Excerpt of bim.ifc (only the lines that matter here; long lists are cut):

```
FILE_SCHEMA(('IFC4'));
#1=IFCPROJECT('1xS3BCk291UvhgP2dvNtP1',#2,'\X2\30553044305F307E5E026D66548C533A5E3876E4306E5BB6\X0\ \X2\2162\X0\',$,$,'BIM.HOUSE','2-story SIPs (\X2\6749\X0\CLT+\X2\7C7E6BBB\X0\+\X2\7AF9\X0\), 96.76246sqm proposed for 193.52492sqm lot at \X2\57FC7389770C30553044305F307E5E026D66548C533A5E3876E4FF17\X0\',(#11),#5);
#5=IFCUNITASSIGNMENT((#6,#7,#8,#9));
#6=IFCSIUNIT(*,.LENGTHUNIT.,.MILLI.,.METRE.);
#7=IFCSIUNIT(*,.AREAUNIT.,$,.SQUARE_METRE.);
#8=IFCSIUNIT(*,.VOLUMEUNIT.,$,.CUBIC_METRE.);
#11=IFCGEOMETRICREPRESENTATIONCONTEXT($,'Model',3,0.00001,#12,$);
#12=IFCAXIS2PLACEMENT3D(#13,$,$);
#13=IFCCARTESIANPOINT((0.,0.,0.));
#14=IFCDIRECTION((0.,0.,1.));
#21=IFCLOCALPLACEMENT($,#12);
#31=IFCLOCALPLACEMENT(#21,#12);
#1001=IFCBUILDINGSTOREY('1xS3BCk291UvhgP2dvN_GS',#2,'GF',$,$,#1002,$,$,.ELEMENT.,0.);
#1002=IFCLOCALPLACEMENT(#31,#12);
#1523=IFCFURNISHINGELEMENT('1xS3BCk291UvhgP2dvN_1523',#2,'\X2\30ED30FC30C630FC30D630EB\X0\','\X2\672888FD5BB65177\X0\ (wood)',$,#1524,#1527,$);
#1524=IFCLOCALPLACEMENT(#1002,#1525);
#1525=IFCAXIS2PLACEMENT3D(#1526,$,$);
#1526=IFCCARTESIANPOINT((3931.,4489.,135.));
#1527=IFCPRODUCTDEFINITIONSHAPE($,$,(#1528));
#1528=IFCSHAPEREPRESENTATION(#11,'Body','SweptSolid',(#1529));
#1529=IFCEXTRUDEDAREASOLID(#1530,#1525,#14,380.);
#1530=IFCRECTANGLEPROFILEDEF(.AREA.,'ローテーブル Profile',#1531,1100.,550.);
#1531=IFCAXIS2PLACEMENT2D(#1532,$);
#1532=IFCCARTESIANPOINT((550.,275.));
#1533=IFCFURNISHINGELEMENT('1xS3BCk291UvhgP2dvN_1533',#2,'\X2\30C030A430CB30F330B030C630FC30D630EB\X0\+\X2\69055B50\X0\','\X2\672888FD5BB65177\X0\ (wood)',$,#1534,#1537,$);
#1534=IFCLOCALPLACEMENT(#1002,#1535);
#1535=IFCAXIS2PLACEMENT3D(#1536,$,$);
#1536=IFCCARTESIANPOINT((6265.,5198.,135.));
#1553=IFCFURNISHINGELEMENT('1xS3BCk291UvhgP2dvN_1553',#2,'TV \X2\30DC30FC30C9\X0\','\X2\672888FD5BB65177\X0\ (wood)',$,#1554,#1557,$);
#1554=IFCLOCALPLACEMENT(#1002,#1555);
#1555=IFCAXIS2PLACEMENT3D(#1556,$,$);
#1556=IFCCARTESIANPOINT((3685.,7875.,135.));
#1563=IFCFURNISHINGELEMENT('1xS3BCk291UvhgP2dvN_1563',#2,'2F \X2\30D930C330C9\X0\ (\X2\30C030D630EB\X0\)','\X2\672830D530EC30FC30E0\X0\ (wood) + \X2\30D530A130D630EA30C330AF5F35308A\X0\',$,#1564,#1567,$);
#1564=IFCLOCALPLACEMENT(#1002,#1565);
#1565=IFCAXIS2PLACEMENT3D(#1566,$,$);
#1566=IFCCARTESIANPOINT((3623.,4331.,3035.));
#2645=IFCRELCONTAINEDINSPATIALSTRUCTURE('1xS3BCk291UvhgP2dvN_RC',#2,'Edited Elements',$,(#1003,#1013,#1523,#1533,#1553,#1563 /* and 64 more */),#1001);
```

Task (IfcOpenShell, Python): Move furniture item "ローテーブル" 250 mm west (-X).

```python
import ifcopenshell
import ifcopenshell.api.geometry
import ifcopenshell.util.placement
import ifcopenshell.util.unit

model = ifcopenshell.open("bim.ifc")
unit_scale = ifcopenshell.util.unit.calculate_unit_scale(model)

item = model.by_id(1523)
matrix = ifcopenshell.util.placement.get_local_placement(item.ObjectPlacement)
matrix[0, 3] -= 0.25 / unit_scale
ifcopenshell.api.geometry.edit_object_placement(model, product=item, matrix=matrix, is_si=False)

print(ifcopenshell.util.placement.get_local_placement(item.ObjectPlacement).round(3) + 0.0)

model.write("bim-out.ifc")
```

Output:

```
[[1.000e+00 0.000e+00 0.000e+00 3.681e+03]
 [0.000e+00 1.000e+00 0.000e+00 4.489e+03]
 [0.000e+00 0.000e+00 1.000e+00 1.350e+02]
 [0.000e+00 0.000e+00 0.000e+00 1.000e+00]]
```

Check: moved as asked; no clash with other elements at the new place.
